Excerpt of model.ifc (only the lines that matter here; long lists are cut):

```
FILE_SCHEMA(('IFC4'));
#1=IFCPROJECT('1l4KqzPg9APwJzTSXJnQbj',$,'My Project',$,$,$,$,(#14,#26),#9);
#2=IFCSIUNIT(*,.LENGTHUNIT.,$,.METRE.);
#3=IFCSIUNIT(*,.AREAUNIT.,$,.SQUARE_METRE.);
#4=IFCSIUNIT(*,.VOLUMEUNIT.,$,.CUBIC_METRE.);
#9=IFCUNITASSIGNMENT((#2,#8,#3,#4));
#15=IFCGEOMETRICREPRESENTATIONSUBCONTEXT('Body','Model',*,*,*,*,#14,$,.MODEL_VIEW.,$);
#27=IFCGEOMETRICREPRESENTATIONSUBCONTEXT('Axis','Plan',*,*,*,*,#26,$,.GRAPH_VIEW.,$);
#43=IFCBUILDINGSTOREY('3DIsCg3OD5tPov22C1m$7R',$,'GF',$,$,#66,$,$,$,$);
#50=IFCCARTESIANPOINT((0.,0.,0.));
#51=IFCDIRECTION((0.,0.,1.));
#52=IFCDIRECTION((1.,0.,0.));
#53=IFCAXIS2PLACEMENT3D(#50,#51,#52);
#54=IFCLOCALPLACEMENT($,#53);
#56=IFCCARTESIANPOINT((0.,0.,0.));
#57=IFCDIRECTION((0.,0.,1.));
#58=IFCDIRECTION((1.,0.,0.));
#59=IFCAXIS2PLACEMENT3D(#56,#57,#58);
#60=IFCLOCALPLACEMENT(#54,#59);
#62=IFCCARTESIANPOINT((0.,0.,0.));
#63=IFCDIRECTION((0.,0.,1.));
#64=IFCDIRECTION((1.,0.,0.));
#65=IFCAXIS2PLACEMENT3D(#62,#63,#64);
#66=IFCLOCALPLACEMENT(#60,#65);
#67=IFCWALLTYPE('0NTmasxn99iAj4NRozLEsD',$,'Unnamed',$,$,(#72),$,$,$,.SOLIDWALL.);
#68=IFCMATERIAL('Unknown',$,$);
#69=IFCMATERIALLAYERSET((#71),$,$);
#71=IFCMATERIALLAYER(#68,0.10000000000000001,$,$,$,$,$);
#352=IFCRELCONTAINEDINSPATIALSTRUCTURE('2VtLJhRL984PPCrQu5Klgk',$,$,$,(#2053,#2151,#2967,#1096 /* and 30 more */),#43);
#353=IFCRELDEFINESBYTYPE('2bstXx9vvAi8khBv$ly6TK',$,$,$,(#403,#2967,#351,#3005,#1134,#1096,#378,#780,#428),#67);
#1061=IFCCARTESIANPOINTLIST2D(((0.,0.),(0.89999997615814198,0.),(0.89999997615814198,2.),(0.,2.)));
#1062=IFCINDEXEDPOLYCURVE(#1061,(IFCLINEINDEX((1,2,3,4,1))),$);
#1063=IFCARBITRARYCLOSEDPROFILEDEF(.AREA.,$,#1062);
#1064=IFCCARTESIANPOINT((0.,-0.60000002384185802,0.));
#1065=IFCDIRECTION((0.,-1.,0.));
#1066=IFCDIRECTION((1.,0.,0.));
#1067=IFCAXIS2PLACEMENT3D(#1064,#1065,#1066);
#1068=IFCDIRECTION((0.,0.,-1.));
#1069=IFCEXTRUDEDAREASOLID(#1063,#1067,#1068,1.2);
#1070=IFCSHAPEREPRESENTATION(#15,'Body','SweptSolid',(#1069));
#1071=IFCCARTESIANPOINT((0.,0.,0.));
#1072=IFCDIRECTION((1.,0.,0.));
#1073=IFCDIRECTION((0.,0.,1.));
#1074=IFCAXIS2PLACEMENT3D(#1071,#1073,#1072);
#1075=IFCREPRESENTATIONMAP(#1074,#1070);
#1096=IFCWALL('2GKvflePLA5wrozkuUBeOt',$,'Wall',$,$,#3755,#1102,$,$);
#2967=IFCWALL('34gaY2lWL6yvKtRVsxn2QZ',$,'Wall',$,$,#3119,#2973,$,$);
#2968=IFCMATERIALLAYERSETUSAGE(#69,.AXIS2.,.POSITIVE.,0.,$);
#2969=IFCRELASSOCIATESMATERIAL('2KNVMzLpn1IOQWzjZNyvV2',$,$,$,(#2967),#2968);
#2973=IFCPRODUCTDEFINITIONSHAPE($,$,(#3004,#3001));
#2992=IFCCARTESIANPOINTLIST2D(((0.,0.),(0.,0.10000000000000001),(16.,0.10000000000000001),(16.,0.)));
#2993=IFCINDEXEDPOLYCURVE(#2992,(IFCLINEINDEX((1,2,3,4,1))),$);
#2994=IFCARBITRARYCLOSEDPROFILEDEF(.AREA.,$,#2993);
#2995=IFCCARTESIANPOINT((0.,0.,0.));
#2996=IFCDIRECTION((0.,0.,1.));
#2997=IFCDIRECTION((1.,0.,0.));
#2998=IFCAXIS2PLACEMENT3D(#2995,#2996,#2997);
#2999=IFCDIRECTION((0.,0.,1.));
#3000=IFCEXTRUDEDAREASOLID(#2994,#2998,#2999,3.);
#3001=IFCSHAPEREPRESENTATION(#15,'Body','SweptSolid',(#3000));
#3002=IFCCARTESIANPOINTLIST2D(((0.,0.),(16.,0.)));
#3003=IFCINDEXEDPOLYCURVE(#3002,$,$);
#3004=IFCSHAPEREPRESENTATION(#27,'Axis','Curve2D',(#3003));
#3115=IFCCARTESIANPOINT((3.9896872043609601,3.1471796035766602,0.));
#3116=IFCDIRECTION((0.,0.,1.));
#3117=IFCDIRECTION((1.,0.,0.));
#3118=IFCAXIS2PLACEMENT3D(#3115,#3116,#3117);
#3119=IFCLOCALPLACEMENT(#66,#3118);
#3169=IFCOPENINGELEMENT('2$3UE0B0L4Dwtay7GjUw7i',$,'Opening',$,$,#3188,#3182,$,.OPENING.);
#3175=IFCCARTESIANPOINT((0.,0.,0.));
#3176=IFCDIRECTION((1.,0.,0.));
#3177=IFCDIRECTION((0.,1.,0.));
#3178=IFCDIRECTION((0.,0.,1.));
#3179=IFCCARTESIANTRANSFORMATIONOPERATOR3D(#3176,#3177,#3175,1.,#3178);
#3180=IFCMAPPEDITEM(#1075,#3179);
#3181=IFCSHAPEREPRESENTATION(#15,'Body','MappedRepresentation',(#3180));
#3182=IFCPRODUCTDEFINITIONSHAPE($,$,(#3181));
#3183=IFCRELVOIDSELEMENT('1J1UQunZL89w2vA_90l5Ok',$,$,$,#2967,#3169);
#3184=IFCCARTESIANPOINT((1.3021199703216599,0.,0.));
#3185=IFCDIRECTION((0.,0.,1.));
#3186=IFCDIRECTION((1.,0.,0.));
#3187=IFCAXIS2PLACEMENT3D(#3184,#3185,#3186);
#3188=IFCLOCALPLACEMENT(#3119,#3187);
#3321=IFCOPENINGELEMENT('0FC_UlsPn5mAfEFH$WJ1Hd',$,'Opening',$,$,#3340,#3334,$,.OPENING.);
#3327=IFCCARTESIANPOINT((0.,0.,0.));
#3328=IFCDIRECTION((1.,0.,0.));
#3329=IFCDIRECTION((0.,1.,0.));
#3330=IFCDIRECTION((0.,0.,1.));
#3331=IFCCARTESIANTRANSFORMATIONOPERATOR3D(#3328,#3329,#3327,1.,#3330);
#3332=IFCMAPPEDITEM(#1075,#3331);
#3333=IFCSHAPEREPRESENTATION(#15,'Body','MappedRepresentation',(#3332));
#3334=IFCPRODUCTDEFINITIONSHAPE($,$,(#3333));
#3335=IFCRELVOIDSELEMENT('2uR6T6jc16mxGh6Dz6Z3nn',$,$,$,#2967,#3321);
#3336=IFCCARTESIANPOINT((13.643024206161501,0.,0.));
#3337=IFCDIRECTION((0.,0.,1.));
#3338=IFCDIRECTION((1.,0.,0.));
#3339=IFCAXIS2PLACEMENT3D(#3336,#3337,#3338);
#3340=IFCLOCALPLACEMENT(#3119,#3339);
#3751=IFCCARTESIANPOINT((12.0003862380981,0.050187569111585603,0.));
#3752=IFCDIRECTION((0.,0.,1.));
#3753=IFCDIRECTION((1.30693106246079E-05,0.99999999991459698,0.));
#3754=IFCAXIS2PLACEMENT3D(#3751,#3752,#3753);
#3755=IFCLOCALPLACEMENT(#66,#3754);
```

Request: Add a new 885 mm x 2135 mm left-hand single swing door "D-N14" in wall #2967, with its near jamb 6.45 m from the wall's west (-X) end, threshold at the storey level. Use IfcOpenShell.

```python
import numpy as np
import ifcopenshell
import ifcopenshell.api.feature
import ifcopenshell.api.geometry
import ifcopenshell.api.root
import ifcopenshell.api.spatial
import ifcopenshell.geom
import ifcopenshell.util.element
import ifcopenshell.util.placement
import ifcopenshell.util.representation
import ifcopenshell.util.shape
import ifcopenshell.util.unit

model = ifcopenshell.open("model.ifc")
unit_scale = ifcopenshell.util.unit.calculate_unit_scale(model)
settings = ifcopenshell.geom.settings()


def volume(element):
    """Net volume in cubic metres, openings subtracted."""
    shape = ifcopenshell.geom.create_shape(settings, element)
    return ifcopenshell.util.shape.get_volume(shape.geometry)


wall = model.by_guid("34gaY2lWL6yvKtRVsxn2QZ")
storey = ifcopenshell.util.element.get_container(wall, ifc_class="IfcBuildingStorey")
context = ifcopenshell.util.representation.get_context(model, "Model", "Body", "MODEL_VIEW")
before = volume(wall)

width, height, from_end, sill = 0.885, 2.135, 6.45, 0.0  # metres

# The wall runs along its own X axis, and the end named is its -X end.
wall_shape = ifcopenshell.geom.create_shape(settings, wall)
x, y, z = ifcopenshell.util.shape.get_vertices(wall_shape.geometry).T
start = x.min() + from_end
face, thickness = float(y.min()), float(y.max() - y.min())
wall_matrix = ifcopenshell.util.placement.get_local_placement(wall.ObjectPlacement)
level = ifcopenshell.util.placement.get_local_placement(storey.ObjectPlacement)[2, 3]


def in_wall(x, y):
    """Placement at x, y metres in the wall's axes, at sill height."""
    matrix = wall_matrix.copy()
    matrix[:, 3] = wall_matrix @ np.array([x / unit_scale, y / unit_scale, 0.0, 1.0])
    matrix[2, 3] = level + sill / unit_scale
    return matrix


# Opening: a box that overshoots both wall faces by 50 mm.
opening = ifcopenshell.api.root.create_entity(model, ifc_class="IfcOpeningElement", predefined_type="OPENING")
box = ifcopenshell.api.geometry.add_wall_representation(
    model, context=context, length=width, height=height, thickness=thickness + 0.1
)
ifcopenshell.api.geometry.assign_representation(model, product=opening, representation=box)
ifcopenshell.api.geometry.edit_object_placement(model, product=opening, matrix=in_wall(start, face - 0.05), is_si=False)
ifcopenshell.api.feature.add_feature(model, feature=opening, element=wall)

door = ifcopenshell.api.root.create_entity(model, ifc_class="IfcDoor", name="D-N14", predefined_type="DOOR")
door.OverallWidth, door.OverallHeight = width / unit_scale, height / unit_scale
door.OperationType = "SINGLE_SWING_LEFT"
body = ifcopenshell.api.geometry.add_door_representation(
    model,
    context=context,
    overall_width=door.OverallWidth,
    overall_height=door.OverallHeight,
    operation_type="SINGLE_SWING_LEFT",
    lining_properties={"LiningDepth": thickness / unit_scale, "ThresholdDepth": thickness / unit_scale},
)
ifcopenshell.api.geometry.assign_representation(model, product=door, representation=body)
ifcopenshell.api.spatial.assign_container(model, products=[door], relating_structure=storey)
ifcopenshell.api.feature.add_filling(model, opening=opening, element=door)

# The lining spans the wall, so the door starts at the wall face.
ifcopenshell.api.geometry.edit_object_placement(model, product=door, matrix=in_wall(start, face), is_si=False)

after = volume(wall)

print(f"wall volume {before:.3f} -> {after:.3f} m3")

model.write("model_edited.ifc")
```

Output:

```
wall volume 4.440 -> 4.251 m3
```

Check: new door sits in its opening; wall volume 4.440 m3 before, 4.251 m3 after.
